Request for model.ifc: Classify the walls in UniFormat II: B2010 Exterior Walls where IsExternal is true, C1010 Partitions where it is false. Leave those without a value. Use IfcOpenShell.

First a look at what the model holds.

```python
import ifcopenshell
import ifcopenshell.util.element

model = ifcopenshell.open("model.ifc")
print(model.schema)
print("classifications:", [c.Name for c in model.by_type("IfcClassification")])
values = [ifcopenshell.util.element.get_pset(e, "Pset_WallCommon", "IsExternal") for e in model.by_type("IfcWall")]
for value in (True, False, None):
    print("IsExternal", value, values.count(value))
```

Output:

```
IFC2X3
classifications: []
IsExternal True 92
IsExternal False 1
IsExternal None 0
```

```python
import ifcopenshell
import ifcopenshell.api.classification
import ifcopenshell.util.element

model = ifcopenshell.open("model.ifc")

# IFC2X3 requires Source and Edition and has no link from the project to the system.
system = model.create_entity("IfcClassification", Source="ASTM", Edition="E1557", Name="UniFormat II")

walls = model.by_type("IfcWall")
external = {e: ifcopenshell.util.element.get_pset(e, "Pset_WallCommon", "IsExternal") for e in walls}
for flag, code, name in ((True, "B2010", "Exterior Walls"), (False, "C1010", "Partitions")):
    products = [e for e in walls if external[e] is flag]
    ifcopenshell.api.classification.add_reference(
        model, products=products, classification=system, identification=code, name=name
    )
    print(code, len(products))

model.write("model_rev.ifc")
```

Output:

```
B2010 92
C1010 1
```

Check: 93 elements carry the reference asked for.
